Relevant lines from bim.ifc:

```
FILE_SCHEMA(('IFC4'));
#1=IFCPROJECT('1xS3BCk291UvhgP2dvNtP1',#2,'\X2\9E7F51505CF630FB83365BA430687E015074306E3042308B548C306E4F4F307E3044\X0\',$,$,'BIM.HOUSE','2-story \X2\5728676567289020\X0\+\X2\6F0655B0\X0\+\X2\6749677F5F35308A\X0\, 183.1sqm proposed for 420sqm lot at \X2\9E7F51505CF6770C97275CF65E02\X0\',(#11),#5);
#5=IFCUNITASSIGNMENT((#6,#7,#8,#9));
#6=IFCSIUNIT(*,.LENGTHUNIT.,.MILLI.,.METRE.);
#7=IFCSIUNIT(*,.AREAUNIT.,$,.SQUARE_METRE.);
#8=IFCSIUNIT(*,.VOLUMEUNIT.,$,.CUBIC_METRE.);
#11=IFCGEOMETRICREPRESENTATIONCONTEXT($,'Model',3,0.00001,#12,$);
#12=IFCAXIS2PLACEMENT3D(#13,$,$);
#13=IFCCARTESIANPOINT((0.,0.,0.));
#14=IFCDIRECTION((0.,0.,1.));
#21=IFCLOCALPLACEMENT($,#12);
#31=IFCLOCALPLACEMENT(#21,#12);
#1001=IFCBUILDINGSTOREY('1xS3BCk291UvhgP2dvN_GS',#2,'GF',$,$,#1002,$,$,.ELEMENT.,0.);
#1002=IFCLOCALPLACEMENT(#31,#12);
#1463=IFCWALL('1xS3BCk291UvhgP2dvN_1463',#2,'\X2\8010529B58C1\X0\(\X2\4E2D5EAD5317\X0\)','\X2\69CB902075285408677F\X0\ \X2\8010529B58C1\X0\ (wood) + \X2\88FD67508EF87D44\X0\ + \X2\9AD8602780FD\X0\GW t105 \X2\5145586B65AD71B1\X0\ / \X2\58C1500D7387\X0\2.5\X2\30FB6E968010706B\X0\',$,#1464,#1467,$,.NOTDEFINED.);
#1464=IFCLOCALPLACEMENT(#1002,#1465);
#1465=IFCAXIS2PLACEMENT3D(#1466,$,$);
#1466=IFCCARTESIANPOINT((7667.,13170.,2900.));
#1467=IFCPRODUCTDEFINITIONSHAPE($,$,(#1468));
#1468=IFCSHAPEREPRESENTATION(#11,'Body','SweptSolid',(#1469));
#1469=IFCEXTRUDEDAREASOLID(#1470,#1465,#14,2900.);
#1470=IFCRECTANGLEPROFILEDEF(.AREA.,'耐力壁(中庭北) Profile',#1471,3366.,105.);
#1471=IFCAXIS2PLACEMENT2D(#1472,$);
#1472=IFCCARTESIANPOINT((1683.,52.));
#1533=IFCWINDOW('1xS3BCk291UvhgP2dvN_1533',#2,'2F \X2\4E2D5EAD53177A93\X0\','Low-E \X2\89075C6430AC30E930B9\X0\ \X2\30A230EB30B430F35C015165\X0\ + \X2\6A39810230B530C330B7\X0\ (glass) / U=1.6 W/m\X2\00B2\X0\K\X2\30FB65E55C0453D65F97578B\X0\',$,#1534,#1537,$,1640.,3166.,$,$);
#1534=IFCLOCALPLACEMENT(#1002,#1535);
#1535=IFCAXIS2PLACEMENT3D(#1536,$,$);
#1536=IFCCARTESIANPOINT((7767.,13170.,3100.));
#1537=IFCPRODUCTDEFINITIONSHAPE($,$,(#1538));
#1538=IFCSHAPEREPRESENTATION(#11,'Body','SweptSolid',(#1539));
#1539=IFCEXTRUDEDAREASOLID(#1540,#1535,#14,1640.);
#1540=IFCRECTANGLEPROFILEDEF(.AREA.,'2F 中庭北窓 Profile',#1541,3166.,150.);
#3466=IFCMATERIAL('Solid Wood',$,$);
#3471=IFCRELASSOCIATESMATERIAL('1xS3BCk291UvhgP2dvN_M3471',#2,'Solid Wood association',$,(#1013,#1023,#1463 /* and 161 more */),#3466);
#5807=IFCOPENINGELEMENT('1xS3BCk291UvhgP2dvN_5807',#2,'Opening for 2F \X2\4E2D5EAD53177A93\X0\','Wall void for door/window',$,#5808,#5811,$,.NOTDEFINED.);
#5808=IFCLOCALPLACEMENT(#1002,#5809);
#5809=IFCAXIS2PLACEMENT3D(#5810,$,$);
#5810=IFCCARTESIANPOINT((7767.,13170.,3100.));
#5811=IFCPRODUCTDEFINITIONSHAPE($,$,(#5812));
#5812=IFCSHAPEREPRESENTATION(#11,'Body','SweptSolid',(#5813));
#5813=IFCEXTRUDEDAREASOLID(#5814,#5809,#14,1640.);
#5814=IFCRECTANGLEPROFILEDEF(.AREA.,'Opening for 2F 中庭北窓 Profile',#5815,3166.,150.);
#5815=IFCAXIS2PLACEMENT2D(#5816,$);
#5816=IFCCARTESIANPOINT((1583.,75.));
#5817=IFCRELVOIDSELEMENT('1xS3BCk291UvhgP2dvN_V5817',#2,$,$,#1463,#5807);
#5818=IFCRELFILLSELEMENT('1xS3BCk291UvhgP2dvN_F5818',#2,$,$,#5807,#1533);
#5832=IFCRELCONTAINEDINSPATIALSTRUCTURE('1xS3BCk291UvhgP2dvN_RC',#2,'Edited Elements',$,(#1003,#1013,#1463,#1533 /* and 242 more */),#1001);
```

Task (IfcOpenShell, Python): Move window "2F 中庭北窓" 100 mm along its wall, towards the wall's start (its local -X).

```python
import ifcopenshell
import ifcopenshell.api.geometry
import ifcopenshell.util.placement
import ifcopenshell.util.unit

model = ifcopenshell.open("bim.ifc")
unit_scale = ifcopenshell.util.unit.calculate_unit_scale(model)

window = model.by_id(1533)
opening = window.FillsVoids[0].RelatingOpeningElement
wall = opening.VoidsElements[0].RelatingBuildingElement

wall_matrix = ifcopenshell.util.placement.get_local_placement(wall.ObjectPlacement)
shift = wall_matrix[:3, 0] * -0.1 / unit_scale
before = ifcopenshell.util.placement.get_local_placement(window.ObjectPlacement)[:3, 3].copy()

# The window is not placed relative to its opening, so move both.
for product in (opening, window):
    matrix = ifcopenshell.util.placement.get_local_placement(product.ObjectPlacement)
    matrix[:3, 3] += shift
    ifcopenshell.api.geometry.edit_object_placement(model, product=product, matrix=matrix, is_si=False)

after = ifcopenshell.util.placement.get_local_placement(window.ObjectPlacement)[:3, 3]
print("window moved by", (after - before).round(3) + 0.0)

model.write("bim-out.ifc")
```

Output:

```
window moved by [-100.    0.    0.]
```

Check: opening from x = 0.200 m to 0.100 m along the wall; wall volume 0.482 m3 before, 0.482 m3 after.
